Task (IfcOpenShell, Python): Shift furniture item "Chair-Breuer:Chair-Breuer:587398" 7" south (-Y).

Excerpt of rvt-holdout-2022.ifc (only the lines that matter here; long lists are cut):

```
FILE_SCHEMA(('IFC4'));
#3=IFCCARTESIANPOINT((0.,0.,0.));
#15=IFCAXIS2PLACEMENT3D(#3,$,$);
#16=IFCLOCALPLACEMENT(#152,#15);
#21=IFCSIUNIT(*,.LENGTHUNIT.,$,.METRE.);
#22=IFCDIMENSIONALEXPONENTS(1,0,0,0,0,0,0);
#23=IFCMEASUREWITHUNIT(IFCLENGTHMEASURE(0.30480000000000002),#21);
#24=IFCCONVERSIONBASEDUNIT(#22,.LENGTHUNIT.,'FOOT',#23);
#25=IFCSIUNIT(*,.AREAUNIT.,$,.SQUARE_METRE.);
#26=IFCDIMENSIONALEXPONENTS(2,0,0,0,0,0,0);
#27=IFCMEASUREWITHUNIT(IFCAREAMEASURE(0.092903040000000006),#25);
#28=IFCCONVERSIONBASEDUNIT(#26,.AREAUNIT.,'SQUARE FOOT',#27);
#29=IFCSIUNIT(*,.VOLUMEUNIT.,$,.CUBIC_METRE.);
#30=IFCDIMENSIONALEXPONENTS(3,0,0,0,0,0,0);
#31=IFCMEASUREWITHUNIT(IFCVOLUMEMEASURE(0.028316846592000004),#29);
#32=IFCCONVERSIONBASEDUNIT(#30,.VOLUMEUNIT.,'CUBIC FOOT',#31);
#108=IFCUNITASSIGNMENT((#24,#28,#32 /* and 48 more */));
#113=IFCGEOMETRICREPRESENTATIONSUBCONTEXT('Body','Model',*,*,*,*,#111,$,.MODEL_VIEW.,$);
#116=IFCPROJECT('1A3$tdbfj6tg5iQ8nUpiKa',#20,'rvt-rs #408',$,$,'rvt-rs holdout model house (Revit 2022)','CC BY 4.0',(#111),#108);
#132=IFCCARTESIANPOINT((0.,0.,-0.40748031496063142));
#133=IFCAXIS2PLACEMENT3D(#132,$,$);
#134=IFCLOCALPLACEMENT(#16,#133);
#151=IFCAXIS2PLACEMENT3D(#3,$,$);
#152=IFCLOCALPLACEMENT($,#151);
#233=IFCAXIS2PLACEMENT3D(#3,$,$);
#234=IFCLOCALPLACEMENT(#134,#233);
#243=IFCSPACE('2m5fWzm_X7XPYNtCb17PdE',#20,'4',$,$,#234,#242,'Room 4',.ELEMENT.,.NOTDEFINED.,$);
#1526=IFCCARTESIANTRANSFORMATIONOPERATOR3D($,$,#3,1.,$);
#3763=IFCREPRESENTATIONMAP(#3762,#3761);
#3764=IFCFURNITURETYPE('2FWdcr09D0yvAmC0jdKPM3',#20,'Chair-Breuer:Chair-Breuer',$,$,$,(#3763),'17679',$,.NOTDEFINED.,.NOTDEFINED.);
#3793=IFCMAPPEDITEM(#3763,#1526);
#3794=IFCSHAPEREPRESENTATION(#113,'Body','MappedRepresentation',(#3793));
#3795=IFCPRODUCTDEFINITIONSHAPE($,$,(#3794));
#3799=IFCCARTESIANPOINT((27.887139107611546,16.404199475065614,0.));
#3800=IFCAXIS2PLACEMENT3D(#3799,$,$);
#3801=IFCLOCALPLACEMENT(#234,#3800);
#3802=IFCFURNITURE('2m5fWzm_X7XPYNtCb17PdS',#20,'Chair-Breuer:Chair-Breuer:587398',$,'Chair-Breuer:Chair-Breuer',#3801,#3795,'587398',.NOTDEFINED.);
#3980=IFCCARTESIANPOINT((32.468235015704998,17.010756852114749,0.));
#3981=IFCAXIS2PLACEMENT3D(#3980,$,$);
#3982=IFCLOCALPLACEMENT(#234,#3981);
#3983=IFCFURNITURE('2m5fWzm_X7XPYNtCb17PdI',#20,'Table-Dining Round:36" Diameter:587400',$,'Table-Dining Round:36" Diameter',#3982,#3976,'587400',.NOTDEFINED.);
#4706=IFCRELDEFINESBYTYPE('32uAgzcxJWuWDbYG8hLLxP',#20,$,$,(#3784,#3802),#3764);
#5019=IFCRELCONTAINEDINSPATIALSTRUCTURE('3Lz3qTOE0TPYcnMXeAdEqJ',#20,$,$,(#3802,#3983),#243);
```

```python
import ifcopenshell
import ifcopenshell.api.geometry
import ifcopenshell.util.placement
import ifcopenshell.util.unit

model = ifcopenshell.open("rvt-holdout-2022.ifc")
unit_scale = ifcopenshell.util.unit.calculate_unit_scale(model)

item = model.by_guid("2m5fWzm_X7XPYNtCb17PdS")
matrix = ifcopenshell.util.placement.get_local_placement(item.ObjectPlacement)
matrix[1, 3] -= 7 * 0.0254 / unit_scale
ifcopenshell.api.geometry.edit_object_placement(model, product=item, matrix=matrix, is_si=False)

print(ifcopenshell.util.placement.get_local_placement(item.ObjectPlacement).round(3) + 0.0)

model.write("rvt-holdout-2022_edited.ifc")
```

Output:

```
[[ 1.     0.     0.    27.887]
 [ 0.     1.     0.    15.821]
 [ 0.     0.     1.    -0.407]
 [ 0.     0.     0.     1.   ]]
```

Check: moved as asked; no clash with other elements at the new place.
